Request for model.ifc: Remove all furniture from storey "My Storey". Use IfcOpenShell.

First a look at what the model holds.

```python
import ifcopenshell
import ifcopenshell.util.element

model = ifcopenshell.open("model.ifc")
print(model.schema)
storey = next(s for s in model.by_type("IfcBuildingStorey") if s.Name == "My Storey")
furniture = [e for e in ifcopenshell.util.element.get_decomposition(storey) if e.is_a("IfcFurnishingElement")]
seen = {}
for e in furniture:
    element_type = ifcopenshell.util.element.get_type(e)
    name = element_type.Name if element_type not in (None, e) else None
    seen[name] = seen.get(name, 0) + 1
for name, count in sorted(seen.items(), key=str):
    print(count, "x", name)
```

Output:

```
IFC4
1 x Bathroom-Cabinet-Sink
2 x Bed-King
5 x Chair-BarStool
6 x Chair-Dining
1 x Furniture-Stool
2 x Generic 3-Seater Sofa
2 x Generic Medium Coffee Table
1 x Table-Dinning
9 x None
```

```python
import ifcopenshell
import ifcopenshell.api.root
import ifcopenshell.util.element

model = ifcopenshell.open("model.ifc")

storey = next(s for s in model.by_type("IfcBuildingStorey") if s.Name == "My Storey")
furniture = [e for e in ifcopenshell.util.element.get_decomposition(storey) if e.is_a("IfcFurnishingElement")]

for e in furniture:
    ifcopenshell.api.root.remove_product(model, product=e)
print(len(furniture), "removed")

model.write("model_rev.ifc")
```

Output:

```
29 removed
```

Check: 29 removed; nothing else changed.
